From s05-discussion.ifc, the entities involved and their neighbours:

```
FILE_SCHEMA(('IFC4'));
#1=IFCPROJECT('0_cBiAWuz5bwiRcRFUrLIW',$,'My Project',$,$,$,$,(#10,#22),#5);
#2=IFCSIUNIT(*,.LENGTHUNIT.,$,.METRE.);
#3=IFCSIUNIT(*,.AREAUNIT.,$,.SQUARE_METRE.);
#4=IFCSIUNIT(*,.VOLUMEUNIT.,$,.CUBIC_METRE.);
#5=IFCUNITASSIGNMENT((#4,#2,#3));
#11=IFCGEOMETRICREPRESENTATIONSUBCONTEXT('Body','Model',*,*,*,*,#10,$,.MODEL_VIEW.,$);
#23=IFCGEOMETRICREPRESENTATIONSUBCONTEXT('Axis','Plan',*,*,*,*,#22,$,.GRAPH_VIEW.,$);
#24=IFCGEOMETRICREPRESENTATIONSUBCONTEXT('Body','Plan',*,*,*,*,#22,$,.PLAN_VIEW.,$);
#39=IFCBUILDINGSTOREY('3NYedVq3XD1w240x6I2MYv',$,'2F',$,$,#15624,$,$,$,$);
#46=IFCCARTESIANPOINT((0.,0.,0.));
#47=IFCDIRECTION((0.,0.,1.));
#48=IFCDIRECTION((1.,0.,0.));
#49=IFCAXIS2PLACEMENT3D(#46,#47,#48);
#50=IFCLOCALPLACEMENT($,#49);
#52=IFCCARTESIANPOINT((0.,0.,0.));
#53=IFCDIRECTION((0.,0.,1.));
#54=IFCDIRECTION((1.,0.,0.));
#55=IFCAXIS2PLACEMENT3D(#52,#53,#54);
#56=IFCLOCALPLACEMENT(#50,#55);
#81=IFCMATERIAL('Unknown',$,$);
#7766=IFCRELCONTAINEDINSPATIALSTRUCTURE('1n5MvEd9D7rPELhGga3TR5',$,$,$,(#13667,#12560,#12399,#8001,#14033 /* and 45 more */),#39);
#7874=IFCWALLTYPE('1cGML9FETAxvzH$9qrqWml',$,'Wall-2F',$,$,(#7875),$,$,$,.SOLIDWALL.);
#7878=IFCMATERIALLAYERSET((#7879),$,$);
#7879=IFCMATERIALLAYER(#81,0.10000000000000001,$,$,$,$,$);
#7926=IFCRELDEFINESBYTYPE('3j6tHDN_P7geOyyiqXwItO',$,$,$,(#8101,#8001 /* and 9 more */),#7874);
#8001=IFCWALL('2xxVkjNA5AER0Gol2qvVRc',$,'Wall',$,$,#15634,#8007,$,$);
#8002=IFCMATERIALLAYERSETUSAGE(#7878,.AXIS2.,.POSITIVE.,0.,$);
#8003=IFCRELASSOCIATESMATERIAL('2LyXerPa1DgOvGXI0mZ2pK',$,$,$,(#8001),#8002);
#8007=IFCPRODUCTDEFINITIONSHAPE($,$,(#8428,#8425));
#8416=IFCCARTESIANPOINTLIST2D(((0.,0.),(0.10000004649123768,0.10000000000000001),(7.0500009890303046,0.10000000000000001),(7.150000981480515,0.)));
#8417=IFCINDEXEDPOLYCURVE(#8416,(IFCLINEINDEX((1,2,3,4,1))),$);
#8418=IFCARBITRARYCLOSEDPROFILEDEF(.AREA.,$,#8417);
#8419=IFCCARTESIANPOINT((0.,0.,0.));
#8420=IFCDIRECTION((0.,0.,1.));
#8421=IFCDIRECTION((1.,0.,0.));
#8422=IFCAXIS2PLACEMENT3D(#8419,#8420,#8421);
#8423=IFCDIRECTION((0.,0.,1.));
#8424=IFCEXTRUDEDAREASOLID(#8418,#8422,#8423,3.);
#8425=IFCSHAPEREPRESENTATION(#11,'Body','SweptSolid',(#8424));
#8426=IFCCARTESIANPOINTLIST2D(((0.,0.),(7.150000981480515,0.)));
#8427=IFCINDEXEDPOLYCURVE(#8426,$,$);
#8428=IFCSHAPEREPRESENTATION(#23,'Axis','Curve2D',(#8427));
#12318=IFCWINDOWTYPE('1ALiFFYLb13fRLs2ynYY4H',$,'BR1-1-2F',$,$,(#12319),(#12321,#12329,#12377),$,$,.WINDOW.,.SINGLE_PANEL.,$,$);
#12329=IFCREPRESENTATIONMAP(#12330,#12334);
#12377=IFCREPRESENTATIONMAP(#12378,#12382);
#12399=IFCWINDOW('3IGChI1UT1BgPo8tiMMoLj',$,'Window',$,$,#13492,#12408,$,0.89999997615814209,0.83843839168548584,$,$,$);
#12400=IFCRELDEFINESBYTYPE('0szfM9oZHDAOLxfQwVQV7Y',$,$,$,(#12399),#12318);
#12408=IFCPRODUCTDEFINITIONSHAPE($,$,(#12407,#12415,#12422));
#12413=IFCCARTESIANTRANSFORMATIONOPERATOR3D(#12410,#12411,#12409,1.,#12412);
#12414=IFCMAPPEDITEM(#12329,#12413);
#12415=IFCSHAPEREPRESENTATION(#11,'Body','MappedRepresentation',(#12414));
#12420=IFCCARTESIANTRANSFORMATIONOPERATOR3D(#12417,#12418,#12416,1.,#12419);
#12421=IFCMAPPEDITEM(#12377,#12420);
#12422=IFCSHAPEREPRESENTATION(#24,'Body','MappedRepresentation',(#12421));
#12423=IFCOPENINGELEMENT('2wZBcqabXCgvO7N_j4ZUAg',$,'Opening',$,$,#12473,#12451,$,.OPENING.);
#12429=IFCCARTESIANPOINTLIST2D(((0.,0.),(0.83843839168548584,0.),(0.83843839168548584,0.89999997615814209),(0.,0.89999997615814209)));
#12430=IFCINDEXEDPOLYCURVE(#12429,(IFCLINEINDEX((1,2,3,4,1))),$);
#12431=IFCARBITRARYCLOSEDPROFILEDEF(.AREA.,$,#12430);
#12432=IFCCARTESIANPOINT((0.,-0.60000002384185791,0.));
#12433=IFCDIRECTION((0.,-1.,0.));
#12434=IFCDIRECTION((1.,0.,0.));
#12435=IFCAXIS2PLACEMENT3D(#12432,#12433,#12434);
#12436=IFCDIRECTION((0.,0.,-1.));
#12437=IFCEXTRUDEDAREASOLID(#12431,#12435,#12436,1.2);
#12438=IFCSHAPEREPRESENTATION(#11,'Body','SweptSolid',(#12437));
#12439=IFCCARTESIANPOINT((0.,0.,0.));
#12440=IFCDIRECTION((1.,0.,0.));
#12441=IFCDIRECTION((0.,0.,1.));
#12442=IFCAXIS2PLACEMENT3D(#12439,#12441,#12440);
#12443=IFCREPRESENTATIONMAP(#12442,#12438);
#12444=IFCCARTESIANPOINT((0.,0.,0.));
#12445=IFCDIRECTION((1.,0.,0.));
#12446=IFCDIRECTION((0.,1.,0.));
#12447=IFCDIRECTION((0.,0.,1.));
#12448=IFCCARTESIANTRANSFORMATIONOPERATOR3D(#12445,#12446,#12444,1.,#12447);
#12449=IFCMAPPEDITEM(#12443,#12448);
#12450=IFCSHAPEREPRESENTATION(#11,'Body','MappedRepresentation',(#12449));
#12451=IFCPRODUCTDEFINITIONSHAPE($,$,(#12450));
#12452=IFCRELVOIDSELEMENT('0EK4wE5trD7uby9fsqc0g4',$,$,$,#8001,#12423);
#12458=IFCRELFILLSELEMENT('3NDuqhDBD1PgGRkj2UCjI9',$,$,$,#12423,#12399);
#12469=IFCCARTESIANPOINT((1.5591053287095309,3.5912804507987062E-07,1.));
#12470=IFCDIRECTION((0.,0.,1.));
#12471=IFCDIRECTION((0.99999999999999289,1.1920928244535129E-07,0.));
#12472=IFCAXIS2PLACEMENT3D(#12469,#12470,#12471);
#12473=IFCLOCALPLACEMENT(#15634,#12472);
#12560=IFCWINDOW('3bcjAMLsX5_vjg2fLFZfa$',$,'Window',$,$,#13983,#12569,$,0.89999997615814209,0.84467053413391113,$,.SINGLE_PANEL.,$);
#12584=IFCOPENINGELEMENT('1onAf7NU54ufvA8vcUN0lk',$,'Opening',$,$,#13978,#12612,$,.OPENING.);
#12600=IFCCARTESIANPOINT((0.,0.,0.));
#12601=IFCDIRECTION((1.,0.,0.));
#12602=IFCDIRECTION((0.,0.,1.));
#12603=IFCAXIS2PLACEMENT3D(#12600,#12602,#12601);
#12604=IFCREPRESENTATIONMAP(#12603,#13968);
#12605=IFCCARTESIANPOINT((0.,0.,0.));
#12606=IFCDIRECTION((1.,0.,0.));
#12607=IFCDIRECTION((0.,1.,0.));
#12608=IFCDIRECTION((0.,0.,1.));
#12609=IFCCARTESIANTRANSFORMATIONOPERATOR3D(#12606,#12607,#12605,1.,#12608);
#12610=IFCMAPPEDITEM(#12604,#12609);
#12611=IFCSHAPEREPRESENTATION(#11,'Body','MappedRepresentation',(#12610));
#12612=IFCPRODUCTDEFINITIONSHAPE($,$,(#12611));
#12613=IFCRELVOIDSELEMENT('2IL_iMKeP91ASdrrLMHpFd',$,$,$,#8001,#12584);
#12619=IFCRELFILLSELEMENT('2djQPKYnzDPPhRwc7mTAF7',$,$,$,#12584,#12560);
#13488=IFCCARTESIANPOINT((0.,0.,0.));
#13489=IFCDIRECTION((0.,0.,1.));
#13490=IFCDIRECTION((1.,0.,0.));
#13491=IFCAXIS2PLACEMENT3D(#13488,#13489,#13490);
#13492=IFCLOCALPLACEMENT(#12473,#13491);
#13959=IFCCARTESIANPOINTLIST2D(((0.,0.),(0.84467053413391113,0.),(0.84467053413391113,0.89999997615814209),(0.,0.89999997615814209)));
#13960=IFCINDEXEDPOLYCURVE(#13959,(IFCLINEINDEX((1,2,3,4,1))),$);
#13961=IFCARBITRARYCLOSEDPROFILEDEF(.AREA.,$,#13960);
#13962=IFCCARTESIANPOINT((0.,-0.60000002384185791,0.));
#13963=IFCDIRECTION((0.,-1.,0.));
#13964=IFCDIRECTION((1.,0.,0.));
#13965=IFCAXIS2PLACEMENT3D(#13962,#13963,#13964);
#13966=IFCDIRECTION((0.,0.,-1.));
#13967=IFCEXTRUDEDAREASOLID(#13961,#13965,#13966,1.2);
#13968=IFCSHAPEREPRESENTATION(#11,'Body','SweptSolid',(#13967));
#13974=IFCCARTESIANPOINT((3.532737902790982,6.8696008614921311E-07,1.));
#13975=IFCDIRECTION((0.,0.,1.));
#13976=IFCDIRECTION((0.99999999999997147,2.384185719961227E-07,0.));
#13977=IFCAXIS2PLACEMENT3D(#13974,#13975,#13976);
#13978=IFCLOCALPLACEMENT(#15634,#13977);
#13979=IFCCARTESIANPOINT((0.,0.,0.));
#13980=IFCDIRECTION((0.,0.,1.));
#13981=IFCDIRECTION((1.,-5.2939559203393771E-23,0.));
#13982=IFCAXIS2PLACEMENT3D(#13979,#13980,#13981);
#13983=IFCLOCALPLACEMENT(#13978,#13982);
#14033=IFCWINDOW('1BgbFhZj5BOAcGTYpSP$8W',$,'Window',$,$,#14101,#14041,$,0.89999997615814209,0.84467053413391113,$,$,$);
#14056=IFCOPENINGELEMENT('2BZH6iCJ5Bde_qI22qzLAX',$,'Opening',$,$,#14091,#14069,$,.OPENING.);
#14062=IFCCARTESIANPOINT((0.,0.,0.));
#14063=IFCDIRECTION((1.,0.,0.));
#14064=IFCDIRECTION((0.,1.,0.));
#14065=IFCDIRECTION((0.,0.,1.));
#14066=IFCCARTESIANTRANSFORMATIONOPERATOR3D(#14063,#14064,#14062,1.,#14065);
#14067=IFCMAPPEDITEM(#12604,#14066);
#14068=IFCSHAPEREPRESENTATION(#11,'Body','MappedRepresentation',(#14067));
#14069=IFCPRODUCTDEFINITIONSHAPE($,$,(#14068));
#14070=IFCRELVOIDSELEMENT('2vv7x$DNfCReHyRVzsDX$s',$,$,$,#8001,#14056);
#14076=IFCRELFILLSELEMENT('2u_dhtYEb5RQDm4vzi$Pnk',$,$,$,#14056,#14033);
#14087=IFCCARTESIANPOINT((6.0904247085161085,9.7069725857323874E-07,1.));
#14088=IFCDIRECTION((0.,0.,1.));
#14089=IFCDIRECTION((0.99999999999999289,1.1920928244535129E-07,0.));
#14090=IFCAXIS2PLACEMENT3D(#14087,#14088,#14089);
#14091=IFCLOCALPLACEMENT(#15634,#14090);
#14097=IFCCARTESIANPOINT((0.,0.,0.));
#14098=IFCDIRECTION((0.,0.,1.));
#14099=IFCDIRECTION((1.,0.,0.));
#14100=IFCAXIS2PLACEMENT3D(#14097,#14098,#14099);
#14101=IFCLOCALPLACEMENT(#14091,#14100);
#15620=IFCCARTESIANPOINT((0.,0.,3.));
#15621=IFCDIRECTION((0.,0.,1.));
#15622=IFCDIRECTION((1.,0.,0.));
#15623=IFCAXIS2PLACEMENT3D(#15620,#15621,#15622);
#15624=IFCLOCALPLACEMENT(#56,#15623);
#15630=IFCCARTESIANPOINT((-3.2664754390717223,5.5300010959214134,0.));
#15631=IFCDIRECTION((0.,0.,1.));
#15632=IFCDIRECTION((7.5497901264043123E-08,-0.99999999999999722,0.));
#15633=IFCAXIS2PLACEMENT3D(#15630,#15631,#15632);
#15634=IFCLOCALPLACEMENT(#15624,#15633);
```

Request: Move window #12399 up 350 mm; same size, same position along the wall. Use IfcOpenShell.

```python
import numpy as np
import ifcopenshell
import ifcopenshell.api.geometry
import ifcopenshell.util.placement
import ifcopenshell.util.unit

model = ifcopenshell.open("s05-discussion.ifc")
unit_scale = ifcopenshell.util.unit.calculate_unit_scale(model)

window = model.by_guid("3IGChI1UT1BgPo8tiMMoLj")
opening = window.FillsVoids[0].RelatingOpeningElement
dz = 0.35 / unit_scale

shift = np.array([0.0, 0.0, dz])
# The window is placed relative to its opening, so it follows when the opening moves.
matrix = ifcopenshell.util.placement.get_local_placement(opening.ObjectPlacement)
matrix[:3, 3] += shift
ifcopenshell.api.geometry.edit_object_placement(
    model, product=opening, matrix=matrix, is_si=False, should_transform_children=True
)

print(f"moved by {dz * unit_scale:+.3f} m")

model.write("s05-discussion-out.ifc")
```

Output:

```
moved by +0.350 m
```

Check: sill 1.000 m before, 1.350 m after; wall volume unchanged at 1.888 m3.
